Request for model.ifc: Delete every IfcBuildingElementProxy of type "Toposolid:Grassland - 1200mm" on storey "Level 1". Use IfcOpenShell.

First a look at what the model holds.

```python
import ifcopenshell
import ifcopenshell.util.element

model = ifcopenshell.open("model.ifc")
print(model.schema)
storey = next(s for s in model.by_type("IfcBuildingStorey") if s.Name == "Level 1")
proxies = [e for e in ifcopenshell.util.element.get_decomposition(storey) if e.is_a("IfcBuildingElementProxy")]
seen = {}
for e in proxies:
    element_type = ifcopenshell.util.element.get_type(e)
    name = element_type.Name if element_type not in (None, e) else None
    seen[name] = seen.get(name, 0) + 1
for name, count in sorted(seen.items(), key=str):
    print(count, "x", name)
```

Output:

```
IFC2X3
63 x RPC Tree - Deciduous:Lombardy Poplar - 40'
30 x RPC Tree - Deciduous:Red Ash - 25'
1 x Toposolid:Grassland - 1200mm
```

```python
import ifcopenshell
import ifcopenshell.api.root
import ifcopenshell.util.element

model = ifcopenshell.open("model.ifc")

storey = next(s for s in model.by_type("IfcBuildingStorey") if s.Name == "Level 1")
proxies = [e for e in ifcopenshell.util.element.get_decomposition(storey) if e.is_a("IfcBuildingElementProxy")]
targets = [e for e in proxies if (t := ifcopenshell.util.element.get_type(e)) not in (None, e) and t.Name == "Toposolid:Grassland - 1200mm"]

for e in targets:
    ifcopenshell.api.root.remove_product(model, product=e)
print(len(targets), "removed")

model.write("model_edited.ifc")
```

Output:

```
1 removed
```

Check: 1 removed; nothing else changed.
